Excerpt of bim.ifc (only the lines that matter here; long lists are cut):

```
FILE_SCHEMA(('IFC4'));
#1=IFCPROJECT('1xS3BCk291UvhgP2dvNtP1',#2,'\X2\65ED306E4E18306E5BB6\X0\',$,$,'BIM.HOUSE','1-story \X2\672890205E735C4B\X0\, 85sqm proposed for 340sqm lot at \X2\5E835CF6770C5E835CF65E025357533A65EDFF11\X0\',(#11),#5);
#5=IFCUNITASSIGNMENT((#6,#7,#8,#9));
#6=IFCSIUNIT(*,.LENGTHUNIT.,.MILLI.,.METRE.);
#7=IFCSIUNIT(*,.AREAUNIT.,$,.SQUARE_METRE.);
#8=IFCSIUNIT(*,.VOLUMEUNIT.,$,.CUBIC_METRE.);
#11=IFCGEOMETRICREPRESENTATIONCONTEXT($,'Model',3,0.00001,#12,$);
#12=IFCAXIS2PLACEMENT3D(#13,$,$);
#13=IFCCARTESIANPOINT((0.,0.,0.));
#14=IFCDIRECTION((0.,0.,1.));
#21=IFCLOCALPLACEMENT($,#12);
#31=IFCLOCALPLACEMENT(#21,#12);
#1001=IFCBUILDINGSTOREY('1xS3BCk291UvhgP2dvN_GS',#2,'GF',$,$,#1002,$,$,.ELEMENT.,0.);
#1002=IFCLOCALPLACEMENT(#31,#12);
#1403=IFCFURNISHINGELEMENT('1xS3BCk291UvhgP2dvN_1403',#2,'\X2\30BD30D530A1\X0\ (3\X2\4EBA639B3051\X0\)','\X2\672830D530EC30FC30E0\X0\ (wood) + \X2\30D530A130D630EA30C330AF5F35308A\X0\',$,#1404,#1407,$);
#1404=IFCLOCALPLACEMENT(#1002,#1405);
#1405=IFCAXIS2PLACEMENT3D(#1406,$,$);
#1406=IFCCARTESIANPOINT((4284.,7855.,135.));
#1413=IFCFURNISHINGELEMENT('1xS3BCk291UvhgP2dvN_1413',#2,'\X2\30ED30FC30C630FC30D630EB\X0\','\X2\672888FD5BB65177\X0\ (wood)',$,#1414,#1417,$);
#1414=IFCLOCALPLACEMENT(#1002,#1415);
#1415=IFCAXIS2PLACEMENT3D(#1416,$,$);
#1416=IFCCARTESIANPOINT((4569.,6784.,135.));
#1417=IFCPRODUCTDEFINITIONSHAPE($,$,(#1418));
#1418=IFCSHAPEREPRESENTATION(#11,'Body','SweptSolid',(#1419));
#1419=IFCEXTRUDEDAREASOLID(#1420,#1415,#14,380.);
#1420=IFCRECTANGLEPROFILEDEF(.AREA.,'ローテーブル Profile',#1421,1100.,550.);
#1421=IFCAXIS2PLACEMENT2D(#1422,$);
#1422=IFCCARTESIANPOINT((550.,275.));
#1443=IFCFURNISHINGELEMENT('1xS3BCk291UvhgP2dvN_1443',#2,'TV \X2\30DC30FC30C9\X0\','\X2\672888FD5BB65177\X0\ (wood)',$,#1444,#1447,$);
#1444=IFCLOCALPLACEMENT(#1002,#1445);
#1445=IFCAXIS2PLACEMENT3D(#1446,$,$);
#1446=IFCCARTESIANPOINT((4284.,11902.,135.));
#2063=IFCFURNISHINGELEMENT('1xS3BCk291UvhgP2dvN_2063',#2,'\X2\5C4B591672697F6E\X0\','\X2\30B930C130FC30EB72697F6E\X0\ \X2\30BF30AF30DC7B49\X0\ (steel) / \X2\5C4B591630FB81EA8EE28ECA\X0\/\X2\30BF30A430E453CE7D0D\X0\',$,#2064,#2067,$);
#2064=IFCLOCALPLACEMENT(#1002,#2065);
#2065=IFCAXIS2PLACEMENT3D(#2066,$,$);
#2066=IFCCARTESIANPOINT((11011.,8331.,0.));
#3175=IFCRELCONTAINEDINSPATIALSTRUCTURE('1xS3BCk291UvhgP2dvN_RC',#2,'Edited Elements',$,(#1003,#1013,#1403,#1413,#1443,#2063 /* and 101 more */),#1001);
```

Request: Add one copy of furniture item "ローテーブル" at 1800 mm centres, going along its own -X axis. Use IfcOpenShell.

```python
import ifcopenshell
import ifcopenshell.api.geometry
import ifcopenshell.api.root
import ifcopenshell.util.element
import ifcopenshell.util.placement
import ifcopenshell.util.unit

model = ifcopenshell.open("bim.ifc")
unit_scale = ifcopenshell.util.unit.calculate_unit_scale(model)


def reuse_history(source, copy):
    """copy_class also copies each property set's owner history, people and application; keep the originals."""
    for rel in copy.IsDefinedBy:
        if rel.is_a("IfcRelDefinesByProperties") and (history := rel.RelatingPropertyDefinition.OwnerHistory):
            rel.RelatingPropertyDefinition.OwnerHistory = source.OwnerHistory
            ifcopenshell.util.element.remove_deep2(model, history)


source = model.by_guid("1xS3BCk291UvhgP2dvN_1413")
base = ifcopenshell.util.placement.get_local_placement(source.ObjectPlacement)
step = -base[:3, 0] * 1.8 / unit_scale

for i in range(1, 2):
    copy = ifcopenshell.api.root.copy_class(model, product=source)
    copy.Representation = ifcopenshell.util.element.copy_deep(
        model, source.Representation, exclude=["IfcGeometricRepresentationContext", "IfcRepresentationMap"]
    )
    reuse_history(source, copy)
    matrix = base.copy()
    matrix[:3, 3] += i * step
    print("added at", matrix[:3, 3].round(3) + 0.0)
    ifcopenshell.api.geometry.edit_object_placement(model, product=copy, matrix=matrix, is_si=False)

model.write("bim_edited.ifc")
```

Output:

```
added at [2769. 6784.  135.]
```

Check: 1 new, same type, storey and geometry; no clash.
